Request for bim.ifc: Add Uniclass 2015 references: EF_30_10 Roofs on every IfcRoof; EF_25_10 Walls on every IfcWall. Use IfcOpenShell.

First a look at what the model holds.

```python
import ifcopenshell

model = ifcopenshell.open("bim.ifc")
print(model.schema)
print("classifications:", [c.Name for c in model.by_type("IfcClassification")])
for ifc_class in ("IfcDoor", "IfcRoof", "IfcStair", "IfcWall", "IfcWindow"):
    print(ifc_class, len(model.by_type(ifc_class)))
```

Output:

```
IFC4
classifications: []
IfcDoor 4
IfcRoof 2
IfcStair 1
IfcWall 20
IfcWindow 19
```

```python
import ifcopenshell
import ifcopenshell.api.classification

model = ifcopenshell.open("bim.ifc")

system = ifcopenshell.api.classification.add_classification(model, classification="Uniclass 2015")

codes = {
    "IfcRoof": ("EF_30_10", "Roofs"),
    "IfcWall": ("EF_25_10", "Walls"),
}
for ifc_class, (code, name) in codes.items():
    products = model.by_type(ifc_class)
    ifcopenshell.api.classification.add_reference(
        model, products=products, classification=system, identification=code, name=name
    )
    print(code, len(products))

model.write("bim_rev.ifc")
```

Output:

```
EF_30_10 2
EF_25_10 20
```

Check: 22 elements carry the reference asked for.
